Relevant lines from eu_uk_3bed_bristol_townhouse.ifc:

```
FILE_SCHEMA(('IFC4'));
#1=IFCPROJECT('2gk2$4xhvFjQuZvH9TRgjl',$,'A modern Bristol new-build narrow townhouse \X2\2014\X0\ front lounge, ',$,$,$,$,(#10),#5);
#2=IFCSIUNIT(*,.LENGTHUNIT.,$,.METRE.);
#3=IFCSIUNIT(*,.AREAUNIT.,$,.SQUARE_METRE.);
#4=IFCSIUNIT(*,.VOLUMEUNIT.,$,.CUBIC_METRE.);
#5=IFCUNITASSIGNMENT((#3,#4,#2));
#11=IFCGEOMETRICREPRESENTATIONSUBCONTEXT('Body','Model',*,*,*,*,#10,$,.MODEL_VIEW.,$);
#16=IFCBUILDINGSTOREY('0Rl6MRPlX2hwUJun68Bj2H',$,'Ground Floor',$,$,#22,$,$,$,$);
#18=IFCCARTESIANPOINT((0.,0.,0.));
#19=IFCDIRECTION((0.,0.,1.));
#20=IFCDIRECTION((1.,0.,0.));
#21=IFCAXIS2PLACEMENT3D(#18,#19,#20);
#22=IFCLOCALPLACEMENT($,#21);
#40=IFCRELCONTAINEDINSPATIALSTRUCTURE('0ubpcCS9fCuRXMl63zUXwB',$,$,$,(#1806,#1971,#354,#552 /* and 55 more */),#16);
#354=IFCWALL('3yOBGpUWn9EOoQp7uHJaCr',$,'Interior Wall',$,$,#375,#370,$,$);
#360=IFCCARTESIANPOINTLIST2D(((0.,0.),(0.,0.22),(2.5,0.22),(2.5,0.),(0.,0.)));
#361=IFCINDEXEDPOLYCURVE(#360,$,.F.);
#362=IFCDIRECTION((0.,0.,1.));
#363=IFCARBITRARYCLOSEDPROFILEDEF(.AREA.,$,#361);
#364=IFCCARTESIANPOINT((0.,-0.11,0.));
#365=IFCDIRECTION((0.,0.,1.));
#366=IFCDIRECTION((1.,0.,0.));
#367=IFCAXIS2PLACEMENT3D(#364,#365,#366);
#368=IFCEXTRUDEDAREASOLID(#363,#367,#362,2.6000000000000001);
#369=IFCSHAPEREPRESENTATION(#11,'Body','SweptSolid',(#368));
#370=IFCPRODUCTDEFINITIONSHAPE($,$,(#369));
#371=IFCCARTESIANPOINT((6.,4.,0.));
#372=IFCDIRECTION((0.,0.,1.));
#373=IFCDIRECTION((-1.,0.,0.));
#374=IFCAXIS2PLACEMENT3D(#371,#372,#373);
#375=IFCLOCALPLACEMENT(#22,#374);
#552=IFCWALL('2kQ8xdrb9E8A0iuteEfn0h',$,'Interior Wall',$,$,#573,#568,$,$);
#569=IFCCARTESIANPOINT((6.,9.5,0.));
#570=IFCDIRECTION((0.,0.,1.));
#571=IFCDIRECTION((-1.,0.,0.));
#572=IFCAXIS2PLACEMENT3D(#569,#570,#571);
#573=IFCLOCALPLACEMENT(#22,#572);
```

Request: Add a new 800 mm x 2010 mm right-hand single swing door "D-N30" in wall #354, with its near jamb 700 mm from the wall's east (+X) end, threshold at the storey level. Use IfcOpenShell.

```python
import numpy as np
import ifcopenshell
import ifcopenshell.api.feature
import ifcopenshell.api.geometry
import ifcopenshell.api.root
import ifcopenshell.api.spatial
import ifcopenshell.geom
import ifcopenshell.util.element
import ifcopenshell.util.placement
import ifcopenshell.util.representation
import ifcopenshell.util.shape
import ifcopenshell.util.unit

model = ifcopenshell.open("eu_uk_3bed_bristol_townhouse.ifc")
unit_scale = ifcopenshell.util.unit.calculate_unit_scale(model)
settings = ifcopenshell.geom.settings()


def volume(element):
    """Net volume in cubic metres, openings subtracted."""
    shape = ifcopenshell.geom.create_shape(settings, element)
    return ifcopenshell.util.shape.get_volume(shape.geometry)


wall = model.by_guid("3yOBGpUWn9EOoQp7uHJaCr")
storey = ifcopenshell.util.element.get_container(wall, ifc_class="IfcBuildingStorey")
context = ifcopenshell.util.representation.get_context(model, "Model", "Body", "MODEL_VIEW")
before = volume(wall)

width, height, from_end, sill = 0.8, 2.01, 0.7, 0.0  # metres

# The wall runs along its own X axis, and the end named is its -X end.
wall_shape = ifcopenshell.geom.create_shape(settings, wall)
x, y, z = ifcopenshell.util.shape.get_vertices(wall_shape.geometry).T
start = x.min() + from_end
face, thickness = float(y.min()), float(y.max() - y.min())
wall_matrix = ifcopenshell.util.placement.get_local_placement(wall.ObjectPlacement)
level = ifcopenshell.util.placement.get_local_placement(storey.ObjectPlacement)[2, 3]


def in_wall(x, y):
    """Placement at x, y metres in the wall's axes, at sill height."""
    matrix = wall_matrix.copy()
    matrix[:, 3] = wall_matrix @ np.array([x / unit_scale, y / unit_scale, 0.0, 1.0])
    matrix[2, 3] = level + sill / unit_scale
    return matrix


# Opening: a box that overshoots both wall faces by 50 mm.
opening = ifcopenshell.api.root.create_entity(model, ifc_class="IfcOpeningElement", predefined_type="OPENING")
box = ifcopenshell.api.geometry.add_wall_representation(
    model, context=context, length=width, height=height, thickness=thickness + 0.1
)
ifcopenshell.api.geometry.assign_representation(model, product=opening, representation=box)
ifcopenshell.api.geometry.edit_object_placement(model, product=opening, matrix=in_wall(start, face - 0.05), is_si=False)
ifcopenshell.api.feature.add_feature(model, feature=opening, element=wall)

door = ifcopenshell.api.root.create_entity(model, ifc_class="IfcDoor", name="D-N30", predefined_type="DOOR")
door.OverallWidth, door.OverallHeight = width / unit_scale, height / unit_scale
door.OperationType = "SINGLE_SWING_RIGHT"
body = ifcopenshell.api.geometry.add_door_representation(
    model,
    context=context,
    overall_width=door.OverallWidth,
    overall_height=door.OverallHeight,
    operation_type="SINGLE_SWING_RIGHT",
    lining_properties={"LiningDepth": thickness / unit_scale, "ThresholdDepth": thickness / unit_scale},
)
ifcopenshell.api.geometry.assign_representation(model, product=door, representation=body)
ifcopenshell.api.spatial.assign_container(model, products=[door], relating_structure=storey)
ifcopenshell.api.feature.add_filling(model, opening=opening, element=door)

# The lining spans the wall, so the door starts at the wall face.
ifcopenshell.api.geometry.edit_object_placement(model, product=door, matrix=in_wall(start, face), is_si=False)

after = volume(wall)

print(f"wall volume {before:.3f} -> {after:.3f} m3")

model.write("eu_uk_3bed_bristol_townhouse-out.ifc")
```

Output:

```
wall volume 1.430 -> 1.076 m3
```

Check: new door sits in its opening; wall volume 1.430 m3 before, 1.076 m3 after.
